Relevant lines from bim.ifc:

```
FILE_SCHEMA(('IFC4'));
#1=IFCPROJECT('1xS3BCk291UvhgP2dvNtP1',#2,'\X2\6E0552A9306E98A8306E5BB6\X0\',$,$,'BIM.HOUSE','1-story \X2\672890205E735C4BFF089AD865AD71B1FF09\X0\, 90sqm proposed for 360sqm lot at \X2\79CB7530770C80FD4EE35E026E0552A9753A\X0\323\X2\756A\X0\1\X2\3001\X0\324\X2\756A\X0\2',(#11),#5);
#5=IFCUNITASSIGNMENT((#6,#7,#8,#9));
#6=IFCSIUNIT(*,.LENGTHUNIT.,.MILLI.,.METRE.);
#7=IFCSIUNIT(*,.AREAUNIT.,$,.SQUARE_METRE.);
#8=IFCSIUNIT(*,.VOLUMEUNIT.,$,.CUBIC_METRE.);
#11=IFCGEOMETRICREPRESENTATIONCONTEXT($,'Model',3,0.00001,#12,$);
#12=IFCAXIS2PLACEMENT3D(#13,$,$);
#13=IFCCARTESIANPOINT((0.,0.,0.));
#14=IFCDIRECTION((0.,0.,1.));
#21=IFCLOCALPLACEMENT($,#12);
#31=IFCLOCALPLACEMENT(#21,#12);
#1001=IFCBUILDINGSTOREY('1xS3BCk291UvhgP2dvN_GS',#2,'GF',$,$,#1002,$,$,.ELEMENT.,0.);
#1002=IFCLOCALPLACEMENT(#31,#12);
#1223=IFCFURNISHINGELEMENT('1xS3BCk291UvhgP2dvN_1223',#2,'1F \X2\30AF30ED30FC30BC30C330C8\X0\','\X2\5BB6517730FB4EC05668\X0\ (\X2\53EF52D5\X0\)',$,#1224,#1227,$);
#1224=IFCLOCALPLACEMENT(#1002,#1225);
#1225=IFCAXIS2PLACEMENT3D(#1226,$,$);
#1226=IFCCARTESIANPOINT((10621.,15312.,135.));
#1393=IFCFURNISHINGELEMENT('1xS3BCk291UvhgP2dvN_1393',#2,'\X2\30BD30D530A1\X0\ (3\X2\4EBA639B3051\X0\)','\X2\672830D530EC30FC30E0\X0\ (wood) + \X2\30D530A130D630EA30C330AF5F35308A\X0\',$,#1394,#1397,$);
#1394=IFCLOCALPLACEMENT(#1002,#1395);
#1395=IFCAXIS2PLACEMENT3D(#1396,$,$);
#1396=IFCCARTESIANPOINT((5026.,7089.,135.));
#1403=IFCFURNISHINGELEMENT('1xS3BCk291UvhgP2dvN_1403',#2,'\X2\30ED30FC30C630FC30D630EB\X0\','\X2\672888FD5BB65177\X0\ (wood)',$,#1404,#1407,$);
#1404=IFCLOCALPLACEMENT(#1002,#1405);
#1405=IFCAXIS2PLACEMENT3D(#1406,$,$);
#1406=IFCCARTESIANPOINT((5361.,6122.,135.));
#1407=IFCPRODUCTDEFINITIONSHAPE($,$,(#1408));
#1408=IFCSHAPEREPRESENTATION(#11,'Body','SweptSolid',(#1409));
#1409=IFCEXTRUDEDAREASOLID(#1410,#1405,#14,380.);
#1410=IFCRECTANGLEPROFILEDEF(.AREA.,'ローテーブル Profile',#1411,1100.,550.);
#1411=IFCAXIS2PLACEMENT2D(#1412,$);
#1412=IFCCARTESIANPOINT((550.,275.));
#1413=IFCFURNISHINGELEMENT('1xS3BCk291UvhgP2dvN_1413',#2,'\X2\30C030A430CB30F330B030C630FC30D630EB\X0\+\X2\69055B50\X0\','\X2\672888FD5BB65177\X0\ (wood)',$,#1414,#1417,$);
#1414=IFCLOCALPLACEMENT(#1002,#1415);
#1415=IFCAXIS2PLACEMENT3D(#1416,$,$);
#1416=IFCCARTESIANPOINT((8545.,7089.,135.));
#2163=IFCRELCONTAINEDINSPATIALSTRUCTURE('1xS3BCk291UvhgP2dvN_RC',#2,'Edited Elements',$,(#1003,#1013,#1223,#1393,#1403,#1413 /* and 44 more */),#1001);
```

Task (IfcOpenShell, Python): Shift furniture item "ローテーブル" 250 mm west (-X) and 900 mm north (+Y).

```python
import ifcopenshell
import ifcopenshell.api.geometry
import ifcopenshell.util.placement

model = ifcopenshell.open("bim.ifc")

item = model.by_id(1403)
matrix = ifcopenshell.util.placement.get_local_placement(item.ObjectPlacement)
matrix[0, 3] -= 250.0
matrix[1, 3] += 900.0
ifcopenshell.api.geometry.edit_object_placement(model, product=item, matrix=matrix, is_si=False)

print(ifcopenshell.util.placement.get_local_placement(item.ObjectPlacement).round(3) + 0.0)

model.write("bim_updated.ifc")
```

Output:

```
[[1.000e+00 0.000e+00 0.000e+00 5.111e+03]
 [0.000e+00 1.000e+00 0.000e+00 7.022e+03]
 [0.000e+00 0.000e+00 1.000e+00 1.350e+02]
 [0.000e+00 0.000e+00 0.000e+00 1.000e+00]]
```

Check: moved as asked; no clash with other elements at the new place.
